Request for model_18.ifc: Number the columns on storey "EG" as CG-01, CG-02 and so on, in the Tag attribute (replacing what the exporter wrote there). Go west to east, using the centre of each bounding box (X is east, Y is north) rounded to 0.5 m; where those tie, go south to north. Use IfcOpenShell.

First a look at what the model holds.

```python
import ifcopenshell
import ifcopenshell.util.element
import ifcopenshell.util.placement

model = ifcopenshell.open("model_18.ifc")
print(model.schema)
storey = next(s for s in model.by_type("IfcBuildingStorey") if s.Name == "EG")
columns = [e for e in ifcopenshell.util.element.get_decomposition(storey) if e.is_a("IfcColumn")]
for e in sorted(columns, key=lambda e: e.id()):
    origin = ifcopenshell.util.placement.get_local_placement(e.ObjectPlacement)[:3, 3]
    print(e.id(), e.Tag, e.Name, origin.round(2) + 0.0, sep=" | ")
```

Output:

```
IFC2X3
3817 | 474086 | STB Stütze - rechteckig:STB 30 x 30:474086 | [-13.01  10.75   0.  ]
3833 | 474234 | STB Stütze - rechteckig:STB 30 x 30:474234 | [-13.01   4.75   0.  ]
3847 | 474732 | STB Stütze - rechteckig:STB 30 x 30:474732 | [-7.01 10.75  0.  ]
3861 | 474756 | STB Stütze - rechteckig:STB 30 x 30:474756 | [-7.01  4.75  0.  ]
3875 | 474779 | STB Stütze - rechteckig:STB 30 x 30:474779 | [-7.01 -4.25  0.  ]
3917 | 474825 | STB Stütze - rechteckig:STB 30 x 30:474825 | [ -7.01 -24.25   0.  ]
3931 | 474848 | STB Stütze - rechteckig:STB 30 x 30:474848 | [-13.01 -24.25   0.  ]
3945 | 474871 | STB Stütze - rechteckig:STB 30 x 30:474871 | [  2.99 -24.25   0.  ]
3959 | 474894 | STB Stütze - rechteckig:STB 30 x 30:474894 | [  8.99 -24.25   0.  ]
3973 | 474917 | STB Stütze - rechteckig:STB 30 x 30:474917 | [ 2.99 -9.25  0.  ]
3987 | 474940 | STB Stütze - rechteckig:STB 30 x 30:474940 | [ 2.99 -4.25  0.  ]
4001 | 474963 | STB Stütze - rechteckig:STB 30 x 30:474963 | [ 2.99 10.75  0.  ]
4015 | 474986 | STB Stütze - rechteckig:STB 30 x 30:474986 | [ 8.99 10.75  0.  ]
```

```python
import ifcopenshell
import ifcopenshell.geom
import ifcopenshell.util.element
import ifcopenshell.util.shape

model = ifcopenshell.open("model_18.ifc")
settings = ifcopenshell.geom.settings()
settings.set("use-world-coords", True)


def centre(element):
    shape = ifcopenshell.geom.create_shape(settings, element)
    return ifcopenshell.util.shape.get_bbox_centroid(shape.geometry)


storey = next(s for s in model.by_type("IfcBuildingStorey") if s.Name == "EG")
columns = [e for e in ifcopenshell.util.element.get_decomposition(storey) if e.is_a("IfcColumn")]

# Insertion points can sit at a corner or the storey origin, so sort by the geometry (in metres).
centres = {e: centre(e) for e in columns}
columns.sort(key=lambda e: (round(centres[e][0] / 0.5), centres[e][1]))

for i, e in enumerate(columns, start=1):
    number = f"CG-{i:02d}"
    e.Tag = number
    print(e.id(), number)

model.write("model_18-out.ifc")
```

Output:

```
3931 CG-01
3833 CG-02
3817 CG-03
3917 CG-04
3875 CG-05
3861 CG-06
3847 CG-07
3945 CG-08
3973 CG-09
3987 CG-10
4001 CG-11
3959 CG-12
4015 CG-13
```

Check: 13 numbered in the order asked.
